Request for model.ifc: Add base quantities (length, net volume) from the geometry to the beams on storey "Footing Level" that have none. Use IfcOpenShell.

First a look at what the model holds.

```python
import ifcopenshell
import ifcopenshell.util.element
import ifcopenshell.util.unit

model = ifcopenshell.open("model.ifc")
print(model.schema)
for unit_type in ("LENGTHUNIT", "AREAUNIT", "VOLUMEUNIT"):
    print(unit_type, ifcopenshell.util.unit.calculate_unit_scale(model, unit_type))
storey = next(s for s in model.by_type("IfcBuildingStorey") if s.Name == "Footing Level")
beams = [e for e in ifcopenshell.util.element.get_decomposition(storey) if e.is_a("IfcBeam")]
for e in sorted(beams, key=lambda e: e.id()):
    print(e.id(), e.is_a(), e.Name, list(ifcopenshell.util.element.get_psets(e, qtos_only=True)), sep=" | ")
```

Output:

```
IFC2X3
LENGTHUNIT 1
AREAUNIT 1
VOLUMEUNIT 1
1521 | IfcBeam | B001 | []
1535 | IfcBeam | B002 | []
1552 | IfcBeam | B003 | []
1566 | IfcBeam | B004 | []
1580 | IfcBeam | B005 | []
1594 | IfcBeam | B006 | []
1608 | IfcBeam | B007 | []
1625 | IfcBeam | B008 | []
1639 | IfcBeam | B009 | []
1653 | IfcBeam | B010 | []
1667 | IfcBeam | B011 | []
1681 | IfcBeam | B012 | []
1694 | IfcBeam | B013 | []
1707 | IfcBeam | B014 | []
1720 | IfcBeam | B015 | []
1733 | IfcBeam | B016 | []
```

```python
import ifcopenshell
import ifcopenshell.api.pset
import ifcopenshell.geom
import ifcopenshell.util.element
import ifcopenshell.util.shape
import ifcopenshell.util.unit

model = ifcopenshell.open("model.ifc")
unit_scale = ifcopenshell.util.unit.calculate_unit_scale(model)
volume_scale = ifcopenshell.util.unit.calculate_unit_scale(model, "VOLUMEUNIT")
settings = ifcopenshell.geom.settings()

storey = next(s for s in model.by_type("IfcBuildingStorey") if s.Name == "Footing Level")
beams = [e for e in ifcopenshell.util.element.get_decomposition(storey) if e.is_a("IfcBeam")]

for e in sorted(beams, key=lambda e: e.id()):
    if ifcopenshell.util.element.get_psets(e, qtos_only=True, should_inherit=False):
        continue
    # Geometry comes back in metres, in the element's own axes.
    shape = ifcopenshell.geom.create_shape(settings, e)
    values = {
        "Length": ifcopenshell.util.shape.get_max_xyz(shape.geometry) / unit_scale,
        "NetVolume": ifcopenshell.util.shape.get_volume(shape.geometry) / volume_scale,
    }
    qto = ifcopenshell.api.pset.add_qto(model, product=e, name="BaseQuantities")
    ifcopenshell.api.pset.edit_qto(model, qto=qto, properties=values)
    print(e.id(), {k: round(v, 3) for k, v in values.items()})

model.write("model_rev.ifc")
```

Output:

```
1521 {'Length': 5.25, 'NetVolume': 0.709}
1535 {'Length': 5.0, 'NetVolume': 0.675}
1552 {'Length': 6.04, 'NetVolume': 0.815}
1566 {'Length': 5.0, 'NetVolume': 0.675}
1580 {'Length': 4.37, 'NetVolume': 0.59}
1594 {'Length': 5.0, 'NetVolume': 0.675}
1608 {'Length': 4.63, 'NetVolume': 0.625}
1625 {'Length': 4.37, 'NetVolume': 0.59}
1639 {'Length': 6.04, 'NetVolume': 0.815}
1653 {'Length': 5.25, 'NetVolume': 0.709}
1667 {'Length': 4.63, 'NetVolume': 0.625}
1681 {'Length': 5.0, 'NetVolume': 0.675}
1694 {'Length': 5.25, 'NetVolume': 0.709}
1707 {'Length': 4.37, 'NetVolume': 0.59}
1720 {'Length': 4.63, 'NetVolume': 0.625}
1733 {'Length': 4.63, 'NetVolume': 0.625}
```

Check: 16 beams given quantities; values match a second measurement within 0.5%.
